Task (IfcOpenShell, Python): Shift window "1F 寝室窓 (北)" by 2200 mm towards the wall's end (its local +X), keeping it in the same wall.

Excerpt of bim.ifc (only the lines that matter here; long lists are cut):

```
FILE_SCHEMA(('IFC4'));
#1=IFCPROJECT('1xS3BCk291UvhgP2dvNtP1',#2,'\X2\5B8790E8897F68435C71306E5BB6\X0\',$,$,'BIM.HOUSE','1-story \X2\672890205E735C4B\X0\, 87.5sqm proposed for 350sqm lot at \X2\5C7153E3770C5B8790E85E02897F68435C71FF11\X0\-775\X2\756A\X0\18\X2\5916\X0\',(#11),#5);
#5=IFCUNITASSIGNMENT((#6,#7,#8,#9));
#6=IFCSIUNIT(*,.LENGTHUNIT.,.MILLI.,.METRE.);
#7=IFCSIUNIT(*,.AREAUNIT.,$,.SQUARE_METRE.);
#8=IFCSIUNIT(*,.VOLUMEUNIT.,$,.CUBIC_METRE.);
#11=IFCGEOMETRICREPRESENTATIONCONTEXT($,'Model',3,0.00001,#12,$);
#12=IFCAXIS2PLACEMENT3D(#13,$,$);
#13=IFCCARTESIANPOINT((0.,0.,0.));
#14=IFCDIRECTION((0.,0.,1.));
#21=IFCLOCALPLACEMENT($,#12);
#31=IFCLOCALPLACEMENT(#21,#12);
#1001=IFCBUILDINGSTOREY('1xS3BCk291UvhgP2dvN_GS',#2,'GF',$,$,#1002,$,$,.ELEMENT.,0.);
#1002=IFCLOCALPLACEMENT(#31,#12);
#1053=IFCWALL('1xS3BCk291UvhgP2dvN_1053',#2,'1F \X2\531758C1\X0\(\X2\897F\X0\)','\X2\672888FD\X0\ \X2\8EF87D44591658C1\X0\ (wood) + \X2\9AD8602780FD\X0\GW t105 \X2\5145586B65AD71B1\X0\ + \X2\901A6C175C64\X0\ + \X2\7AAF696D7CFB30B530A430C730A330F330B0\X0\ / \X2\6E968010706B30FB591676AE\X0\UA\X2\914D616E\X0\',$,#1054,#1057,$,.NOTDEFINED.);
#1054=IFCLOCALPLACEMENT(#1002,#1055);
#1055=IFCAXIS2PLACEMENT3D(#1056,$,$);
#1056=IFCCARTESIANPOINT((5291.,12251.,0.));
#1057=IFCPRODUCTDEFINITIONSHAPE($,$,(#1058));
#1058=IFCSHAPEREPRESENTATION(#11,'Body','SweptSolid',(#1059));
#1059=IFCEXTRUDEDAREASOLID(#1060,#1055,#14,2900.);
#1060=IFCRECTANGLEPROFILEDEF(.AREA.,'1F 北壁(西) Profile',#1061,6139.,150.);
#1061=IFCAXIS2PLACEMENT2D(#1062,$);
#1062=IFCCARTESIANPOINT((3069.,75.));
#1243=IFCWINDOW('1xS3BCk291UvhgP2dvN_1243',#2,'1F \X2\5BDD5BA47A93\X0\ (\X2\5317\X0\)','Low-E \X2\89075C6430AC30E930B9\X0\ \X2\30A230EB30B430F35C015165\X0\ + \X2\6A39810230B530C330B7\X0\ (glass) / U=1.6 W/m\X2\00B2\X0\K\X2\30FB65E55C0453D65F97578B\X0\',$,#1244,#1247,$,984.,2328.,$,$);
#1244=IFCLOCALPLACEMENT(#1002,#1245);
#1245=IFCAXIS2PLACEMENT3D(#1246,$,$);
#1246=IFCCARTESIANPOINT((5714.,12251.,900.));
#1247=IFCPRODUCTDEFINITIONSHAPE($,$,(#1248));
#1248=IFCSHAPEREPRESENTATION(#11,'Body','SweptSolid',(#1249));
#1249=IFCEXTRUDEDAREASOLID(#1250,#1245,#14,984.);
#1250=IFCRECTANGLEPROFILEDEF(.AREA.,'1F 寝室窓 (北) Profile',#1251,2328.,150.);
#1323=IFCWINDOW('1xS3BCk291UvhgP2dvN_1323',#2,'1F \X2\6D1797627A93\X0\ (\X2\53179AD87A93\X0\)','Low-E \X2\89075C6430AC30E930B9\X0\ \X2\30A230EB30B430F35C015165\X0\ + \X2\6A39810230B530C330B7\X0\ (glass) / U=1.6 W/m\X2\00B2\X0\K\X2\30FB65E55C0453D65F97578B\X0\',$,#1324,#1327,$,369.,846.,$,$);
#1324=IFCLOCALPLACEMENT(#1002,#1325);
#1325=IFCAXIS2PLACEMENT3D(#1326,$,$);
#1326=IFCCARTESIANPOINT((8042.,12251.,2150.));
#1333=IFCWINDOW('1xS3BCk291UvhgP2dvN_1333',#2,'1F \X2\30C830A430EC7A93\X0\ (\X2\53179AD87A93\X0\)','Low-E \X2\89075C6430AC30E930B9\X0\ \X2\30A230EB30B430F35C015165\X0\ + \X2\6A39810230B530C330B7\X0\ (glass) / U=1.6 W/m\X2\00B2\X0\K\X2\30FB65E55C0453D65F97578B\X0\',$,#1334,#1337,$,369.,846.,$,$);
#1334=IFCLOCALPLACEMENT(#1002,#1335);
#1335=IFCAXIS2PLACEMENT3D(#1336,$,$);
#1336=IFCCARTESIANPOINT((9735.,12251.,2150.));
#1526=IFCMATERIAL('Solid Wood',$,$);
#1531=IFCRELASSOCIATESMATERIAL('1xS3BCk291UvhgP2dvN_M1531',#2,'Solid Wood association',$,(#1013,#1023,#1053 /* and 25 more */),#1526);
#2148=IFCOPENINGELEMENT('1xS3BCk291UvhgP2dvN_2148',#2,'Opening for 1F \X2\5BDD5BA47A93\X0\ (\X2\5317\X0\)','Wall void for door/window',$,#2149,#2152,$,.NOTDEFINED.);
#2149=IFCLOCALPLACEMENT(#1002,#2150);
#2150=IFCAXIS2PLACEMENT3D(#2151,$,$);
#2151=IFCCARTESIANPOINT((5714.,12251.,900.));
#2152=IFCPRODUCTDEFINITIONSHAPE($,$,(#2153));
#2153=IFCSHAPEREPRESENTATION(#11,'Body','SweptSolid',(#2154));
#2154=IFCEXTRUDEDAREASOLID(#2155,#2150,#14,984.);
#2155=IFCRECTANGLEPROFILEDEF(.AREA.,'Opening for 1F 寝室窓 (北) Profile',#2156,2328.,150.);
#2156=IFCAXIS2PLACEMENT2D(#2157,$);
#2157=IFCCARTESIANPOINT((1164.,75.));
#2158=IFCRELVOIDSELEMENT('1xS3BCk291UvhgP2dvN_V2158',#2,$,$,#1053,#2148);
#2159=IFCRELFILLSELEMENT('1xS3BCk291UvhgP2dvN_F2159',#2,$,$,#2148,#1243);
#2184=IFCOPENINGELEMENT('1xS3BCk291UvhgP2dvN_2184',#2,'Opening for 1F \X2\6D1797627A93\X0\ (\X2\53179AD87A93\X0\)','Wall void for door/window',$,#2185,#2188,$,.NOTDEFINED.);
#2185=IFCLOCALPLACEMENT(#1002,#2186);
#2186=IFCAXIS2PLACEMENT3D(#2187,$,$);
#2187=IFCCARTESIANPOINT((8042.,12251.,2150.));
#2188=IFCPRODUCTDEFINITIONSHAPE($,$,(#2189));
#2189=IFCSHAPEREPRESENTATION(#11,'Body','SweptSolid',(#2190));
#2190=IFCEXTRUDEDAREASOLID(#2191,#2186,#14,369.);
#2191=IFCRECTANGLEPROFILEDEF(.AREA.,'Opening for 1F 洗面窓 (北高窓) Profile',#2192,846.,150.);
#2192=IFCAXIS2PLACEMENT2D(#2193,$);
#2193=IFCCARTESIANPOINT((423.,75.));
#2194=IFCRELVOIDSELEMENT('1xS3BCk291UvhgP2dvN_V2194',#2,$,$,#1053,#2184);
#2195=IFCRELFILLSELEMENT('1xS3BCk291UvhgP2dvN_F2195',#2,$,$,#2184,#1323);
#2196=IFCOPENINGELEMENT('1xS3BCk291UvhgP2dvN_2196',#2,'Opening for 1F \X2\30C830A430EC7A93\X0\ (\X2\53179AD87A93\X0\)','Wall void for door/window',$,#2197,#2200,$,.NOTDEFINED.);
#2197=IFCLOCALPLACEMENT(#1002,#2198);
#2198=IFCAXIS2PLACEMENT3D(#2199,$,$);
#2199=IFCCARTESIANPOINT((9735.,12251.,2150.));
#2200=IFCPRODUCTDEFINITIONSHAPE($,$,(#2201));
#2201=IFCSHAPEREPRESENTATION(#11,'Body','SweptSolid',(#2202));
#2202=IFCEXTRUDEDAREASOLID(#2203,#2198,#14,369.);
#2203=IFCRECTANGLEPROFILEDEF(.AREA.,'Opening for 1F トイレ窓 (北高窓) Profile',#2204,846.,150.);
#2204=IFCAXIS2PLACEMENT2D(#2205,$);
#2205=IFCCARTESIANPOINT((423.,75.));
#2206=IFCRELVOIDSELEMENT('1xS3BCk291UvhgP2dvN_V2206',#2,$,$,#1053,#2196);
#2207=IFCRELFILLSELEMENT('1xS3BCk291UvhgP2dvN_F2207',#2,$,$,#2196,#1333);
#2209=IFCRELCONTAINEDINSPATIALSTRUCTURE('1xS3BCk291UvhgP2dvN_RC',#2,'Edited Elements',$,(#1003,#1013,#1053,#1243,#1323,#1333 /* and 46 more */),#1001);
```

```python
import ifcopenshell
import ifcopenshell.api.geometry
import ifcopenshell.util.placement

model = ifcopenshell.open("bim.ifc")

window = model.by_id(1243)
opening = window.FillsVoids[0].RelatingOpeningElement
wall = opening.VoidsElements[0].RelatingBuildingElement

wall_matrix = ifcopenshell.util.placement.get_local_placement(wall.ObjectPlacement)
shift = wall_matrix[:3, 0] * 2200.0
before = ifcopenshell.util.placement.get_local_placement(window.ObjectPlacement)[:3, 3].copy()

# The window is not placed relative to its opening, so move both.
for product in (opening, window):
    matrix = ifcopenshell.util.placement.get_local_placement(product.ObjectPlacement)
    matrix[:3, 3] += shift
    ifcopenshell.api.geometry.edit_object_placement(model, product=product, matrix=matrix, is_si=False)

after = ifcopenshell.util.placement.get_local_placement(window.ObjectPlacement)[:3, 3]
print("window moved by", (after - before).round(3) + 0.0)

model.write("bim_rev.ifc")
```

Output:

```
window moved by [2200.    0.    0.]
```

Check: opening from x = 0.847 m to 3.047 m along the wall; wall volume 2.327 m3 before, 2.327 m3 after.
